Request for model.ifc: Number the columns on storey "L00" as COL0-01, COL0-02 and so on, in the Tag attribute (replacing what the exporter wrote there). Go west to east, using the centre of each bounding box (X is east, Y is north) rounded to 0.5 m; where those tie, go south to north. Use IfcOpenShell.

First a look at what the model holds.

```python
import ifcopenshell
import ifcopenshell.util.element
import ifcopenshell.util.placement

model = ifcopenshell.open("model.ifc")
print(model.schema)
storey = next(s for s in model.by_type("IfcBuildingStorey") if s.Name == "L00")
columns = [e for e in ifcopenshell.util.element.get_decomposition(storey) if e.is_a("IfcColumn")]
for e in sorted(columns, key=lambda e: e.id()):
    origin = ifcopenshell.util.placement.get_local_placement(e.ObjectPlacement)[:3, 3]
    print(e.id(), e.Tag, e.Name, origin.round(2) + 0.0, sep=" | ")
```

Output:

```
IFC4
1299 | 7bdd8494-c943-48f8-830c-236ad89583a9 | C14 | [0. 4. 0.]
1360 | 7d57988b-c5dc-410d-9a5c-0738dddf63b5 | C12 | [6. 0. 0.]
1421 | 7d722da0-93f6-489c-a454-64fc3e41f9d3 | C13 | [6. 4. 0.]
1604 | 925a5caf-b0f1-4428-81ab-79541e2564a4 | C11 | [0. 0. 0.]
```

```python
import ifcopenshell
import ifcopenshell.geom
import ifcopenshell.util.element
import ifcopenshell.util.shape

model = ifcopenshell.open("model.ifc")
settings = ifcopenshell.geom.settings()
settings.set("use-world-coords", True)


def centre(element):
    shape = ifcopenshell.geom.create_shape(settings, element)
    return ifcopenshell.util.shape.get_bbox_centroid(shape.geometry)


storey = next(s for s in model.by_type("IfcBuildingStorey") if s.Name == "L00")
columns = [e for e in ifcopenshell.util.element.get_decomposition(storey) if e.is_a("IfcColumn")]

# Insertion points can sit at a corner or the storey origin, so sort by the geometry (in metres).
centres = {e: centre(e) for e in columns}
columns.sort(key=lambda e: (round(centres[e][0] / 0.5), centres[e][1]))

for i, e in enumerate(columns, start=1):
    number = f"COL0-{i:02d}"
    e.Tag = number
    print(e.id(), number)

model.write("model_updated.ifc")
```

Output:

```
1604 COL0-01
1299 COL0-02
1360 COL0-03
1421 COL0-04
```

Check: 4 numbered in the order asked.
